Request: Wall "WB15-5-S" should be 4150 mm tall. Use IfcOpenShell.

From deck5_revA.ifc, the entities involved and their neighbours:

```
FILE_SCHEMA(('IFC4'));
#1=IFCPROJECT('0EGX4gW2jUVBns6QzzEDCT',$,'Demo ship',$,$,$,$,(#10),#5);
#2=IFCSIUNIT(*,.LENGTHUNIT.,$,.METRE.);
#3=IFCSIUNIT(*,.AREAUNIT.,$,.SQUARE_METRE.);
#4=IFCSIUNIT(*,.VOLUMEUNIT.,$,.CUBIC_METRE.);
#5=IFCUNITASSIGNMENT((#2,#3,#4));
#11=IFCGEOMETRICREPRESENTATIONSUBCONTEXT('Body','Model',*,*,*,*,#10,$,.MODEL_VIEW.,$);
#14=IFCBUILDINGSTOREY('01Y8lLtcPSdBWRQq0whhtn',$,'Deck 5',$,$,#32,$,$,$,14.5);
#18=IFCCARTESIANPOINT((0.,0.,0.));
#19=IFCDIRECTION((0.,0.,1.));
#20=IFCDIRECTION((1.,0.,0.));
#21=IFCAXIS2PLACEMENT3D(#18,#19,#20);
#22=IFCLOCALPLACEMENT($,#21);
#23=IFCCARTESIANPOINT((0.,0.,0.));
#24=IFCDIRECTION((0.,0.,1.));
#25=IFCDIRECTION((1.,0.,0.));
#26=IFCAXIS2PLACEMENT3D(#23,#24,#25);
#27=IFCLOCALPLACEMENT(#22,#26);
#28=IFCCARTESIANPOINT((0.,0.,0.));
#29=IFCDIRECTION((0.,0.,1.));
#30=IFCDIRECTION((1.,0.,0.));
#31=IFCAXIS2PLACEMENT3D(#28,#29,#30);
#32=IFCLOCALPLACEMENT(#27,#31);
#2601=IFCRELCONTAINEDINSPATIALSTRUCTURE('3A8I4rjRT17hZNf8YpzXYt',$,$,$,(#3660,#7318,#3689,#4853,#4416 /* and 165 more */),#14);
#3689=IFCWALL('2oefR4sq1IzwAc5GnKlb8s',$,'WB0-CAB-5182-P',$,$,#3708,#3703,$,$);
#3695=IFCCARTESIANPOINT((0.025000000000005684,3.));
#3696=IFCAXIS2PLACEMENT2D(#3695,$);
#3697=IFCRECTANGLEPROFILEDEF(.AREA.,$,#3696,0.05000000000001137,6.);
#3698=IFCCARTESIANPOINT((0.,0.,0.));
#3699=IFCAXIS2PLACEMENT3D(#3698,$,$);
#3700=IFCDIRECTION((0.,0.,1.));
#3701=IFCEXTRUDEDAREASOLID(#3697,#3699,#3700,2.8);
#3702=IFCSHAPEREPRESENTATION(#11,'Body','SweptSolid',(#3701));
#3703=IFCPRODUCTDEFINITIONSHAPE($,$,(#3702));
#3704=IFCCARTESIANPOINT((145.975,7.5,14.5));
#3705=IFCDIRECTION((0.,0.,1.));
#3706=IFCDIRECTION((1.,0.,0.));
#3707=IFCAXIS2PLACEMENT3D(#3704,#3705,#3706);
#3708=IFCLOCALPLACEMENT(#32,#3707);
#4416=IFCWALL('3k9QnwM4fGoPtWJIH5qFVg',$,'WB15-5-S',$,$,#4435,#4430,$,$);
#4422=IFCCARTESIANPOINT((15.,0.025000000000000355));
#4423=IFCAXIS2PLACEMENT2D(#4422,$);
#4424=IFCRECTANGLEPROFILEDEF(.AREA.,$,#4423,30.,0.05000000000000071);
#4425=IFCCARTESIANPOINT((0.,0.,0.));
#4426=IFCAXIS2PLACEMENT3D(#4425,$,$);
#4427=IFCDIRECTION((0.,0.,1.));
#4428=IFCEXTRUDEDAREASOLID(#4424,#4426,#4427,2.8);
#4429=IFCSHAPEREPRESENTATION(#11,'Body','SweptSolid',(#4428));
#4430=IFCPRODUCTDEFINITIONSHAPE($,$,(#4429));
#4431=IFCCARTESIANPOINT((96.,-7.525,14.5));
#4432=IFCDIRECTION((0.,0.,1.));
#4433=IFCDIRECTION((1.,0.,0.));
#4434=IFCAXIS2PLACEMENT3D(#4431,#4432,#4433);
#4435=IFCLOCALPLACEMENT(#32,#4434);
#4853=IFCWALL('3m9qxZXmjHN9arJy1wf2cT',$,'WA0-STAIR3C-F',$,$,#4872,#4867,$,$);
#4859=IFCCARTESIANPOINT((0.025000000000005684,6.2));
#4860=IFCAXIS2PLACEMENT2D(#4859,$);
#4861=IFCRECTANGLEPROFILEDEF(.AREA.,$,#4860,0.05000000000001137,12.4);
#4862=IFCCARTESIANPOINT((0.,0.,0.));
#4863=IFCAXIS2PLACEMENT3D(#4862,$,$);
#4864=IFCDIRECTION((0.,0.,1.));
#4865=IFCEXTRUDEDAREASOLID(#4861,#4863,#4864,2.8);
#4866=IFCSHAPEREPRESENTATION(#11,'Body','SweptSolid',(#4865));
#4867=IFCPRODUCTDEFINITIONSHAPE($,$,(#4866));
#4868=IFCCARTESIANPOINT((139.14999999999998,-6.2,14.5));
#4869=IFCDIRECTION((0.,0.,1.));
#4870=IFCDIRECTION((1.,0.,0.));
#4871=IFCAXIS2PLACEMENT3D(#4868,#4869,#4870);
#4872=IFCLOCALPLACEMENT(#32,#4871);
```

```python
import ifcopenshell
import ifcopenshell.geom
import ifcopenshell.util.representation
import ifcopenshell.util.shape
import ifcopenshell.util.unit

model = ifcopenshell.open("deck5_revA.ifc")
unit_scale = ifcopenshell.util.unit.calculate_unit_scale(model)
settings = ifcopenshell.geom.settings()


def volume(element):
    """Net volume in cubic metres, openings subtracted."""
    shape = ifcopenshell.geom.create_shape(settings, element)
    return ifcopenshell.util.shape.get_volume(shape.geometry)


wall = model.by_guid("3k9QnwM4fGoPtWJIH5qFVg")
before = volume(wall)

body = ifcopenshell.util.representation.get_representation(wall, "Model", "Body")
solid = body.Items[0]
old_height = solid.Depth
solid.Depth = 4.15 / unit_scale
after = volume(wall)

print(f"height {old_height:g} -> {solid.Depth:g}, volume {before:.3f} -> {after:.3f} m3")

model.write("deck5_revA_edited.ifc")
```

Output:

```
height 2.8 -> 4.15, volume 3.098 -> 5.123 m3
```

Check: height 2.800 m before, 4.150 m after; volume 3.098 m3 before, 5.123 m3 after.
